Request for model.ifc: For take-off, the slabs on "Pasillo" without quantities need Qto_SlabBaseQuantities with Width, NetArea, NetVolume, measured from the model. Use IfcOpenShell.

First a look at what the model holds.

```python
import ifcopenshell
import ifcopenshell.util.element
import ifcopenshell.util.unit

model = ifcopenshell.open("model.ifc")
print(model.schema)
for unit_type in ("LENGTHUNIT", "AREAUNIT", "VOLUMEUNIT"):
    print(unit_type, ifcopenshell.util.unit.calculate_unit_scale(model, unit_type))
storey = next(s for s in model.by_type("IfcBuildingStorey") if s.Name == "Pasillo")
slabs = [e for e in ifcopenshell.util.element.get_decomposition(storey) if e.is_a("IfcSlab")]
for e in sorted(slabs, key=lambda e: e.id()):
    print(e.id(), e.is_a(), e.Name, list(ifcopenshell.util.element.get_psets(e, qtos_only=True)), sep=" | ")
```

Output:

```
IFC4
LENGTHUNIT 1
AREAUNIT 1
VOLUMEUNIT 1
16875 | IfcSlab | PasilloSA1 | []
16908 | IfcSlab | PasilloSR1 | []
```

```python
import ifcopenshell
import ifcopenshell.api.pset
import ifcopenshell.geom
import ifcopenshell.util.element
import ifcopenshell.util.shape
import ifcopenshell.util.unit

model = ifcopenshell.open("model.ifc")
unit_scale = ifcopenshell.util.unit.calculate_unit_scale(model)
area_scale = ifcopenshell.util.unit.calculate_unit_scale(model, "AREAUNIT")
volume_scale = ifcopenshell.util.unit.calculate_unit_scale(model, "VOLUMEUNIT")
settings = ifcopenshell.geom.settings()

storey = next(s for s in model.by_type("IfcBuildingStorey") if s.Name == "Pasillo")
slabs = [e for e in ifcopenshell.util.element.get_decomposition(storey) if e.is_a("IfcSlab")]

for e in sorted(slabs, key=lambda e: e.id()):
    if ifcopenshell.util.element.get_psets(e, qtos_only=True, should_inherit=False):
        continue
    # Geometry comes back in metres, in the element's own axes.
    shape = ifcopenshell.geom.create_shape(settings, e)
    values = {
        "Width": ifcopenshell.util.shape.get_z(shape.geometry) / unit_scale,
        "NetArea": ifcopenshell.util.shape.get_footprint_area(shape.geometry) / area_scale,
        "NetVolume": ifcopenshell.util.shape.get_volume(shape.geometry) / volume_scale,
    }
    qto = ifcopenshell.api.pset.add_qto(model, product=e, name="Qto_SlabBaseQuantities")
    ifcopenshell.api.pset.edit_qto(model, qto=qto, properties=values)
    print(e.id(), {k: round(v, 3) for k, v in values.items()})

model.write("model_updated.ifc")
```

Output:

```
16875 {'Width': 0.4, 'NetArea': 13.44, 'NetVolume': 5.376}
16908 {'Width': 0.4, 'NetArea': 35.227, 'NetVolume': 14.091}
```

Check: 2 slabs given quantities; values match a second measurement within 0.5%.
